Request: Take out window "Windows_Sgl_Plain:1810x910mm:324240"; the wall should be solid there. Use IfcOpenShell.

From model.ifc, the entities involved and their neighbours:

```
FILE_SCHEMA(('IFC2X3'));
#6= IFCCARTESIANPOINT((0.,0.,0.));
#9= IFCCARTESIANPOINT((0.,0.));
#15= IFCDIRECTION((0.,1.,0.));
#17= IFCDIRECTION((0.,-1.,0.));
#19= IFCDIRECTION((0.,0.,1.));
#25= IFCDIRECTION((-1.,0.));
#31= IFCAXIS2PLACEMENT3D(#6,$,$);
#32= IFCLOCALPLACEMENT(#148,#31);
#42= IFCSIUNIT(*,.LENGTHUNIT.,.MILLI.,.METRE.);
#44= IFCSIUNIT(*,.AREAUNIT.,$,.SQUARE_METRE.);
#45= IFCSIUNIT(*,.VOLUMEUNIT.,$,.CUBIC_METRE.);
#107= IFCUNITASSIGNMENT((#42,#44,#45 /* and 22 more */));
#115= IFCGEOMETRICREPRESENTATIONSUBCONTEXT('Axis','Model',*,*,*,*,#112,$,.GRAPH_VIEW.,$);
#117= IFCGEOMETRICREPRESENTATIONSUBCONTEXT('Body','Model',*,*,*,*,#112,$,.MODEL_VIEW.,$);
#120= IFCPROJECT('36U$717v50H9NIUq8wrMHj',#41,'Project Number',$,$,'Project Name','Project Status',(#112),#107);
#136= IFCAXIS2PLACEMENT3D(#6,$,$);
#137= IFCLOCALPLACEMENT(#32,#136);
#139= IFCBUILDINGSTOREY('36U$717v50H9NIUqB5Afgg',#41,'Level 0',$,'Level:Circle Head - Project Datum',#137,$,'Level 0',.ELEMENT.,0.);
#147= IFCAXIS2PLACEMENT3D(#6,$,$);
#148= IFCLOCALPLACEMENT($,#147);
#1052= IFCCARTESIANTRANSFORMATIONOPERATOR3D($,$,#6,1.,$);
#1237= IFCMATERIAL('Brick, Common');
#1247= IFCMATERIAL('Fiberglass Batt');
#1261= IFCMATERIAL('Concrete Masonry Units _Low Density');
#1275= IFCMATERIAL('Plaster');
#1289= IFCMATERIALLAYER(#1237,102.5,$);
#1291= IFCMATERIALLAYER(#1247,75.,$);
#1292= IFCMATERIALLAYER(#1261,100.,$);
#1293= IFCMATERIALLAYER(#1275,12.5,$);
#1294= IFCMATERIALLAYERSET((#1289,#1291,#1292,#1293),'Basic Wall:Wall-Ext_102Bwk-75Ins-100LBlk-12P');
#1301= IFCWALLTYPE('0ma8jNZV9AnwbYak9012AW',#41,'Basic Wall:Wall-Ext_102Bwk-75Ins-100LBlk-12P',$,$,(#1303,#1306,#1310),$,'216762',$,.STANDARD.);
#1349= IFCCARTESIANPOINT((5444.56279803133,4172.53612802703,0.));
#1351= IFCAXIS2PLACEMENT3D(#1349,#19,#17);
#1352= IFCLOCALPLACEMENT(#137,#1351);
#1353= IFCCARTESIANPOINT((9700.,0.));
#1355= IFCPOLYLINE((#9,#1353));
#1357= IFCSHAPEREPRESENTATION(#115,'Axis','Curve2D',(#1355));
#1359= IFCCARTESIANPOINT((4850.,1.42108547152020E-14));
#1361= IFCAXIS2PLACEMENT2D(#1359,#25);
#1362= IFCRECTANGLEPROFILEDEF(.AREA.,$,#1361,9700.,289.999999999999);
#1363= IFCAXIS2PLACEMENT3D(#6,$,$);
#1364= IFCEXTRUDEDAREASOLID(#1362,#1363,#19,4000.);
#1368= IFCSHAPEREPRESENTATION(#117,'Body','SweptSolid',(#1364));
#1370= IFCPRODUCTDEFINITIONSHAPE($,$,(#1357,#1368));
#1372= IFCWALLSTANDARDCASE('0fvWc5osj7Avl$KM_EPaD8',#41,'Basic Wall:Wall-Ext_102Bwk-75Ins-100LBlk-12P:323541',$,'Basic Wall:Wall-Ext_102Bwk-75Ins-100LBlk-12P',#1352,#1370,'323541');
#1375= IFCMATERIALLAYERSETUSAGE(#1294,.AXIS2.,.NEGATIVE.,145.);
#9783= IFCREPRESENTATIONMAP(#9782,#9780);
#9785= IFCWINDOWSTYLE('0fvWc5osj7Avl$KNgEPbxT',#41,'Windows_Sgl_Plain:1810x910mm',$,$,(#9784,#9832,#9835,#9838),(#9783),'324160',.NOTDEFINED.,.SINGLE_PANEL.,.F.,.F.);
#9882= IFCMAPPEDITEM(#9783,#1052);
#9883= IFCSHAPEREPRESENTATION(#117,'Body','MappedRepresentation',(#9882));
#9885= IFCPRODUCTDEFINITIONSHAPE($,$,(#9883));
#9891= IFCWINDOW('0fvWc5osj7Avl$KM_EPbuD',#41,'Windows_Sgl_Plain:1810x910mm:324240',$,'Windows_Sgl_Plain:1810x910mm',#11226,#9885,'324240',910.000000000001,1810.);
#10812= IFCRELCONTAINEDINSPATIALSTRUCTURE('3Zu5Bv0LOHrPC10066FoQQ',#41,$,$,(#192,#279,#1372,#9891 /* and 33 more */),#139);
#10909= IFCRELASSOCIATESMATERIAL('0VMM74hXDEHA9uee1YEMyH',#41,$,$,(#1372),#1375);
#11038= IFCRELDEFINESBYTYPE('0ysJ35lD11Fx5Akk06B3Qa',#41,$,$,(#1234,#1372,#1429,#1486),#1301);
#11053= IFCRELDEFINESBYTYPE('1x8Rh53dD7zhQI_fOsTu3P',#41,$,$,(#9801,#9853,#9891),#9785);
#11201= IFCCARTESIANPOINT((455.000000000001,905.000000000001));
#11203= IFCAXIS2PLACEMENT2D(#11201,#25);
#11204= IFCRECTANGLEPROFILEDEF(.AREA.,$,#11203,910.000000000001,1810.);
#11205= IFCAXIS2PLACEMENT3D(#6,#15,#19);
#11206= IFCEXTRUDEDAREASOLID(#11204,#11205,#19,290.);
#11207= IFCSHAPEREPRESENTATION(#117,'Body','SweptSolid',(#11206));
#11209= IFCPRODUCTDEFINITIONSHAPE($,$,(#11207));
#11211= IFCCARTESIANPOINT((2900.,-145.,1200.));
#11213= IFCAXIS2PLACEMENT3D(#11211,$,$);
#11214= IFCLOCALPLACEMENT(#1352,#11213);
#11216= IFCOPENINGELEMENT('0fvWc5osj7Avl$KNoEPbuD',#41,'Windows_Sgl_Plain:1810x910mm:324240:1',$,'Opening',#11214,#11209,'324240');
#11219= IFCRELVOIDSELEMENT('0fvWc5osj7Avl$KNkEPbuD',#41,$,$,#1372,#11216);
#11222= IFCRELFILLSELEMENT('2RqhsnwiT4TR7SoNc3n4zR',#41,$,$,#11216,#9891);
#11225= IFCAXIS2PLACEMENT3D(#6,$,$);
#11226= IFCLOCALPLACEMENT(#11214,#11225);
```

```python
import ifcopenshell
import ifcopenshell.api.feature
import ifcopenshell.api.root
import ifcopenshell.geom
import ifcopenshell.util.shape

model = ifcopenshell.open("model.ifc")
settings = ifcopenshell.geom.settings()


def volume(element):
    """Net volume in cubic metres, openings subtracted."""
    shape = ifcopenshell.geom.create_shape(settings, element)
    return ifcopenshell.util.shape.get_volume(shape.geometry)


window = model.by_guid("0fvWc5osj7Avl$KM_EPbuD")
opening = window.FillsVoids[0].RelatingOpeningElement
wall = opening.VoidsElements[0].RelatingBuildingElement
before = volume(wall)

ifcopenshell.api.root.remove_product(model, product=window)
ifcopenshell.api.feature.remove_feature(model, feature=opening)

after = volume(wall)

print(f"wall volume {before:.3f} -> {after:.3f} m3")

model.write("model_rev.ifc")
```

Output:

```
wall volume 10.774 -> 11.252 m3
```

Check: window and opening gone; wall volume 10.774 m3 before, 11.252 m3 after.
